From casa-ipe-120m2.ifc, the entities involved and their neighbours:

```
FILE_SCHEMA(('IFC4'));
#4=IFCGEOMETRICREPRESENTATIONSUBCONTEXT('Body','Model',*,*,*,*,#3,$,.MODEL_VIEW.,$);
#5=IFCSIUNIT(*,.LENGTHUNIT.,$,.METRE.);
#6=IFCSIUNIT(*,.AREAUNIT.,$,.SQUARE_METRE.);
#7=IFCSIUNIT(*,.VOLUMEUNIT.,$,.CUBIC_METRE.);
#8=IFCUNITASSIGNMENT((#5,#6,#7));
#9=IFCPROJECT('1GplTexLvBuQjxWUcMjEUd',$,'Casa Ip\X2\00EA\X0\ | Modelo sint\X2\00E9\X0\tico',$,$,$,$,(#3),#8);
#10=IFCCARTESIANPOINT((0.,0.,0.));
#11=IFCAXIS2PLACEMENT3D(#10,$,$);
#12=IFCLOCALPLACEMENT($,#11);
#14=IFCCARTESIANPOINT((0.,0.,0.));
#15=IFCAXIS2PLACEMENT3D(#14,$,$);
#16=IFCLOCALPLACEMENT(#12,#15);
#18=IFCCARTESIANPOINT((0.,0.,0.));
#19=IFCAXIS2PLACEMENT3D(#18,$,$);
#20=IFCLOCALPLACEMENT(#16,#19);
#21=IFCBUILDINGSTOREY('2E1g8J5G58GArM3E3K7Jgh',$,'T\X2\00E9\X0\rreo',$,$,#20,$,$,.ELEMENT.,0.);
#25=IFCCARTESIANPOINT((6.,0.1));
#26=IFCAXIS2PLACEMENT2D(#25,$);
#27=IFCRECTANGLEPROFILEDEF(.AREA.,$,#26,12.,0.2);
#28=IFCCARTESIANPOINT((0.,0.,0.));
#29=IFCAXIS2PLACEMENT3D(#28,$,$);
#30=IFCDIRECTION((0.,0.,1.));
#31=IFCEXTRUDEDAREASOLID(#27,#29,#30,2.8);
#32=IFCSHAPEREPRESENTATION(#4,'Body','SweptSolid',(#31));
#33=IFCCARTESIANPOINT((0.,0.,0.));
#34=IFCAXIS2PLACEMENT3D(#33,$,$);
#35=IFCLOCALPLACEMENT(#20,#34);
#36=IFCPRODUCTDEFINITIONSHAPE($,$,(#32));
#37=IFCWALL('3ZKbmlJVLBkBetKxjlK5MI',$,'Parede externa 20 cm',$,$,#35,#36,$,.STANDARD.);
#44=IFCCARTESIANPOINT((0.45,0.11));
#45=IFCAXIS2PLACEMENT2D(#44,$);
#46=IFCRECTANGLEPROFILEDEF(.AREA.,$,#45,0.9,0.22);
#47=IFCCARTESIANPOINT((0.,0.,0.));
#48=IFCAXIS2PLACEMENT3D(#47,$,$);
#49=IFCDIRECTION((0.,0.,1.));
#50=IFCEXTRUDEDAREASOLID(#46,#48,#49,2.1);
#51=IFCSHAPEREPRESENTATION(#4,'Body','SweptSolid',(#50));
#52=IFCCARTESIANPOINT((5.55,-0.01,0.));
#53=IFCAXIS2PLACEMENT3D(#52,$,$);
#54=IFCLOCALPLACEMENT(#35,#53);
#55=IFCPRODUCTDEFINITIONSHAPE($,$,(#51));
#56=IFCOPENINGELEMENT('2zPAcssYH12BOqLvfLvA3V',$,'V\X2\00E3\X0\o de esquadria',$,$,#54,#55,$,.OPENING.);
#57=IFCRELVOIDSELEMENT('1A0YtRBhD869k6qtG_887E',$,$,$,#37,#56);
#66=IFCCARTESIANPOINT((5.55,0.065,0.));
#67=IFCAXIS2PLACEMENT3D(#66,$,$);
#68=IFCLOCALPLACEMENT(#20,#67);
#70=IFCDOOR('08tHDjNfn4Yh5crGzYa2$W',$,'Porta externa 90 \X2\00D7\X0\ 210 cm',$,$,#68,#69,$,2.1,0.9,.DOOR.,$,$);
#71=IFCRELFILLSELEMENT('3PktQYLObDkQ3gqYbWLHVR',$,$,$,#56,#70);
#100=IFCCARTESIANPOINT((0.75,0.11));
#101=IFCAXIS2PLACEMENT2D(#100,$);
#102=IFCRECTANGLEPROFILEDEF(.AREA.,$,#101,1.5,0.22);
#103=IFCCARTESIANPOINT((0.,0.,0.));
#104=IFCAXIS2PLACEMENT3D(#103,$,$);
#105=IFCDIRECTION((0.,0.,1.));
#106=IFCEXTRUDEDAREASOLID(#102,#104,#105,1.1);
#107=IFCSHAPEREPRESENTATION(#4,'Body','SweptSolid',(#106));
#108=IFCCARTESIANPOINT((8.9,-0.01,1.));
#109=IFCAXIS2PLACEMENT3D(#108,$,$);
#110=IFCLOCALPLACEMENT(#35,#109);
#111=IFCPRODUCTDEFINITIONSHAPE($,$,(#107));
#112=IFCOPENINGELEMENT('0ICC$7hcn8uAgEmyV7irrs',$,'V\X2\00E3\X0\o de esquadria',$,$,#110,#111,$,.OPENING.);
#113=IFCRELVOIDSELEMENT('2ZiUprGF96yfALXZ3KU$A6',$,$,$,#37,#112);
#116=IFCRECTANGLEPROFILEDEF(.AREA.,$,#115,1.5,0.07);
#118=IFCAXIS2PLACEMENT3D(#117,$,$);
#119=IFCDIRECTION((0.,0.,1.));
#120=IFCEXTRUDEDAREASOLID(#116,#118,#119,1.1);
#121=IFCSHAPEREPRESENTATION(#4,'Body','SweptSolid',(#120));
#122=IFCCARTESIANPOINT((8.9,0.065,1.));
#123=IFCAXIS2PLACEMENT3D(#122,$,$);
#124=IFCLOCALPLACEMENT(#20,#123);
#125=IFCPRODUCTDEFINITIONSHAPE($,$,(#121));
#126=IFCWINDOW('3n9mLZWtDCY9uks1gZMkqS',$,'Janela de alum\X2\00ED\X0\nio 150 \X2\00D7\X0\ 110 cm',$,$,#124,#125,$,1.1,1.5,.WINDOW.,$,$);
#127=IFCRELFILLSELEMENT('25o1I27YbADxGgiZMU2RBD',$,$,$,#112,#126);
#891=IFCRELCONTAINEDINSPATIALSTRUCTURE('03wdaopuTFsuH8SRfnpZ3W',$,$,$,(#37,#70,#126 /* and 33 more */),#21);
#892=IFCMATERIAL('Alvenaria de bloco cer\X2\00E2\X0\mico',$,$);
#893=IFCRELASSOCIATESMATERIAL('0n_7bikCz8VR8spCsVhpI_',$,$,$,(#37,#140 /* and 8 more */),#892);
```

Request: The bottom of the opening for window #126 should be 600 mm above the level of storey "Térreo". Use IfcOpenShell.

```python
import numpy as np
import ifcopenshell
import ifcopenshell.api.geometry
import ifcopenshell.geom
import ifcopenshell.util.element
import ifcopenshell.util.placement
import ifcopenshell.util.shape
import ifcopenshell.util.unit

model = ifcopenshell.open("casa-ipe-120m2.ifc")
unit_scale = ifcopenshell.util.unit.calculate_unit_scale(model)

window = model.by_id(126)
opening = window.FillsVoids[0].RelatingOpeningElement
storey = ifcopenshell.util.element.get_container(window, ifc_class="IfcBuildingStorey")
level = ifcopenshell.util.placement.get_local_placement(storey.ObjectPlacement)[2, 3]

# The opening's origin need not be at the sill, so measure its lowest point.
shape = ifcopenshell.geom.create_shape(ifcopenshell.geom.settings(), opening)
bottom = ifcopenshell.util.shape.get_shape_bottom_elevation(shape, shape.geometry) / unit_scale
dz = level + 0.6 / unit_scale - bottom

shift = np.array([0.0, 0.0, dz])
# The window is not placed relative to its opening, so move both.
for product in (opening, window):
    matrix = ifcopenshell.util.placement.get_local_placement(product.ObjectPlacement)
    matrix[:3, 3] += shift
    ifcopenshell.api.geometry.edit_object_placement(model, product=product, matrix=matrix, is_si=False)

print(f"moved by {dz * unit_scale:+.3f} m")

model.write("casa-ipe-120m2_updated.ifc")
```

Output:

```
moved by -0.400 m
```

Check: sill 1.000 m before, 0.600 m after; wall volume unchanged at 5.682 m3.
